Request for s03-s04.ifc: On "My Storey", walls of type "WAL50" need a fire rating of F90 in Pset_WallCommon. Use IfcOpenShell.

First a look at what the model holds.

```python
import ifcopenshell
import ifcopenshell.util.element

model = ifcopenshell.open("s03-s04.ifc")
print(model.schema)
storey = next(s for s in model.by_type("IfcBuildingStorey") if s.Name == "My Storey")
walls = [e for e in ifcopenshell.util.element.get_decomposition(storey) if e.is_a("IfcWall")]
seen = {}
for e in walls:
    element_type = ifcopenshell.util.element.get_type(e)
    key = (element_type.Name if element_type != e and element_type else None, ifcopenshell.util.element.get_pset(e, "Pset_WallCommon", "FireRating"))
    seen[key] = seen.get(key, 0) + 1
for (name, value), count in sorted(seen.items(), key=str):
    print(count, "x", name, "|", value)
```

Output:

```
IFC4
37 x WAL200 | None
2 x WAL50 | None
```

```python
import ifcopenshell
import ifcopenshell.api.pset
import ifcopenshell.util.element

model = ifcopenshell.open("s03-s04.ifc")

storey = next(s for s in model.by_type("IfcBuildingStorey") if s.Name == "My Storey")
walls = [e for e in ifcopenshell.util.element.get_decomposition(storey) if e.is_a("IfcWall")]

count = 0
for e in walls:
    element_type = ifcopenshell.util.element.get_type(e)
    if element_type in (None, e) or element_type.Name != "WAL50":
        continue
    # add_pset returns the element's existing set when there is one.
    pset = ifcopenshell.api.pset.add_pset(model, product=e, name="Pset_WallCommon")
    ifcopenshell.api.pset.edit_pset(model, pset=pset, properties={"FireRating": "F90"})
    count += 1

print(count, "walls updated")

model.write("s03-s04_v2.ifc")
```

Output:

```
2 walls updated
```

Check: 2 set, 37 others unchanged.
